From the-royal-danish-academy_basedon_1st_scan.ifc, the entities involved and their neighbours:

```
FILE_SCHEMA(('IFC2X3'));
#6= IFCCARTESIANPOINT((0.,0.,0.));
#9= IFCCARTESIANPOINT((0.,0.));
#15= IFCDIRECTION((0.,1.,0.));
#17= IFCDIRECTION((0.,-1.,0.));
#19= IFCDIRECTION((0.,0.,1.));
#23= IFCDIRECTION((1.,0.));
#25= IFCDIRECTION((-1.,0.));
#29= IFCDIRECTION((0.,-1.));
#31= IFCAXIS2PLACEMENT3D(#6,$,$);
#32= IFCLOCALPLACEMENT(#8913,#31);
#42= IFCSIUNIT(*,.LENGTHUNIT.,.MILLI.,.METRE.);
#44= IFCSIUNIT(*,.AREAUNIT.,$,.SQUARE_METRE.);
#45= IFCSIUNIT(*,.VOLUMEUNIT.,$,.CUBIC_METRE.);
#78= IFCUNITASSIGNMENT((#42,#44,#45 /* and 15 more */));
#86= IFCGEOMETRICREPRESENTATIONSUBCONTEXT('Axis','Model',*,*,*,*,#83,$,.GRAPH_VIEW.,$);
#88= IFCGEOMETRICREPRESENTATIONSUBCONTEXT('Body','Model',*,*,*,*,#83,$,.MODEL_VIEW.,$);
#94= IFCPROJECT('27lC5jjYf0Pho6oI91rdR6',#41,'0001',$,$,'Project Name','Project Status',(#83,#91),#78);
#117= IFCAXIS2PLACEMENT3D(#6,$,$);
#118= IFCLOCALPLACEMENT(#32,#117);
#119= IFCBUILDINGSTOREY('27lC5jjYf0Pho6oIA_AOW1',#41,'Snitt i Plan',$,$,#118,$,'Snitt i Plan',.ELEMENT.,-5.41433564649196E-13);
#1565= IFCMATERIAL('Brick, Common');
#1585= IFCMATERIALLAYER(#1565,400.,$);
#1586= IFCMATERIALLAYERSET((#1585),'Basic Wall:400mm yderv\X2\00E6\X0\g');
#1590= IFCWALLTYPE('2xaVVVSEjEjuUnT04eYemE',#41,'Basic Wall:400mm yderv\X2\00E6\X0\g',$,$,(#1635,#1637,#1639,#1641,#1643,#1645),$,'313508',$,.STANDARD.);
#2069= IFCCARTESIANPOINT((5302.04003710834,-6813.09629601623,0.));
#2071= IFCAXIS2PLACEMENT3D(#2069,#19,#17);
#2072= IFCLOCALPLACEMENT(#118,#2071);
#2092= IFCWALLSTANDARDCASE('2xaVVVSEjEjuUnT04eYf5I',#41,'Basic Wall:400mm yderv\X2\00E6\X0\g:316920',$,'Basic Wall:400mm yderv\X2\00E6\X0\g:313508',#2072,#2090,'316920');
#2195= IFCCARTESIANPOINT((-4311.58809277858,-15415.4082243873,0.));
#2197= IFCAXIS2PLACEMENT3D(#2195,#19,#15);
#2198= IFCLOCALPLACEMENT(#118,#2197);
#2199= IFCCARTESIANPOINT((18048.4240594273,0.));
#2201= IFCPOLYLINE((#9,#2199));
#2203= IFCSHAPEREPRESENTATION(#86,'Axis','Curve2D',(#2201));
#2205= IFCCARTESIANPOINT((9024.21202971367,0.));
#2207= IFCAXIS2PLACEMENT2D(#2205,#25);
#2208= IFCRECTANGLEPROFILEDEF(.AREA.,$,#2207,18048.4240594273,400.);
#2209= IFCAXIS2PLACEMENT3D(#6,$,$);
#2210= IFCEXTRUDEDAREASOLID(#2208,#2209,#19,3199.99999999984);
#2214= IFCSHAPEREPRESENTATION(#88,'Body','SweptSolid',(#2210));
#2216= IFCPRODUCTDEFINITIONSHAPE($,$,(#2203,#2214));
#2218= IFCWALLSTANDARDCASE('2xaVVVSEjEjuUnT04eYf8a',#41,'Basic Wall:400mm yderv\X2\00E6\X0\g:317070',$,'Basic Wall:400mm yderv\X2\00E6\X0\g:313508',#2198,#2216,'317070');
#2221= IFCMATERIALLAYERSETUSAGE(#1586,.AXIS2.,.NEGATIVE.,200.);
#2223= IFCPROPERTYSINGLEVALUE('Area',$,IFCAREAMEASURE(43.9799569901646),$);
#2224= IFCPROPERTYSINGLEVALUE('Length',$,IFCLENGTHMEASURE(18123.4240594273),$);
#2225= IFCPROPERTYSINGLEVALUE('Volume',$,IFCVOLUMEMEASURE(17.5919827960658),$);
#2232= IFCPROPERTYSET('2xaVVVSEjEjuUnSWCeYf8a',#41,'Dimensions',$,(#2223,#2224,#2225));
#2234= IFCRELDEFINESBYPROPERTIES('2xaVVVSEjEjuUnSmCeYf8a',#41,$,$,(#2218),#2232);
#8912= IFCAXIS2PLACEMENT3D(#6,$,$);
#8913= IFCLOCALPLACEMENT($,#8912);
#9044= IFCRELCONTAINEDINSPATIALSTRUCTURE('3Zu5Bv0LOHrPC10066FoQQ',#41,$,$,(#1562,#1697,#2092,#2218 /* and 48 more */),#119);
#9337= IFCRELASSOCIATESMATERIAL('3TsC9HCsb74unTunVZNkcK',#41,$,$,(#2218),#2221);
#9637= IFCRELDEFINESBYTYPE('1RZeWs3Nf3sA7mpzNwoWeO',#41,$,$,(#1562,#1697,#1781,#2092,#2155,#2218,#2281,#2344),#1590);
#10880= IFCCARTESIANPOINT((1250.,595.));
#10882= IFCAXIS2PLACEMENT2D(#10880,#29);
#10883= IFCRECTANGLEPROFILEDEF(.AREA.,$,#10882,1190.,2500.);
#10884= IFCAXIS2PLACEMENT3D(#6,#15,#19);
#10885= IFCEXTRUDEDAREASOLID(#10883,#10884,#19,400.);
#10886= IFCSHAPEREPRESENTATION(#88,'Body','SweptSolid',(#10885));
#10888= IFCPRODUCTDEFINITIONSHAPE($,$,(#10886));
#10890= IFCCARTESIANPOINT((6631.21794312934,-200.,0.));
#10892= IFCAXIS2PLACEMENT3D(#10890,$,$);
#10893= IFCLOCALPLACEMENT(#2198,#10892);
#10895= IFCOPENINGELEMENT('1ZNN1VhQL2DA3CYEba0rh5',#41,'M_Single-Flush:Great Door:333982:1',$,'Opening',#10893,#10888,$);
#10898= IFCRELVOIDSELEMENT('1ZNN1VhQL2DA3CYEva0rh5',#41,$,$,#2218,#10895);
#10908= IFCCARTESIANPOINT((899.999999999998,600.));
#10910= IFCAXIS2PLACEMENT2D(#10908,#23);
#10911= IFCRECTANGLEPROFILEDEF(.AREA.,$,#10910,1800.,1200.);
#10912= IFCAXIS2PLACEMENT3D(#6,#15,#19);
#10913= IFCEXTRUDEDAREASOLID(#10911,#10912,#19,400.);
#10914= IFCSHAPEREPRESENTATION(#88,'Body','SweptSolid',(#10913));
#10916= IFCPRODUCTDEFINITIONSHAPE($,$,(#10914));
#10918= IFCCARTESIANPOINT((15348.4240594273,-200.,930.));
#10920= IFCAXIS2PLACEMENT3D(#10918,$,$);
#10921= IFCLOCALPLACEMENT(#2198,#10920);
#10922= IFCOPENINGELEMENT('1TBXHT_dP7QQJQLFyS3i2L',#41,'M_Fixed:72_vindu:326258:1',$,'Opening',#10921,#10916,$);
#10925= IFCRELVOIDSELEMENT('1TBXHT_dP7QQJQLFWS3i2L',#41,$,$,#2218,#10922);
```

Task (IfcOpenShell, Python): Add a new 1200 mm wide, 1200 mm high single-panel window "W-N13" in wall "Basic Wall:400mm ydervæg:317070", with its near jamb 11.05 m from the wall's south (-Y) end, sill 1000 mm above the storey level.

```python
import numpy as np
import ifcopenshell
import ifcopenshell.api.feature
import ifcopenshell.api.geometry
import ifcopenshell.api.pset
import ifcopenshell.api.root
import ifcopenshell.api.spatial
import ifcopenshell.api.type
import ifcopenshell.geom
import ifcopenshell.util.element
import ifcopenshell.util.placement
import ifcopenshell.util.representation
import ifcopenshell.util.shape
import ifcopenshell.util.unit

model = ifcopenshell.open("the-royal-danish-academy_basedon_1st_scan.ifc")
unit_scale = ifcopenshell.util.unit.calculate_unit_scale(model)
area_scale = ifcopenshell.util.unit.calculate_unit_scale(model, "AREAUNIT")
volume_scale = ifcopenshell.util.unit.calculate_unit_scale(model, "VOLUMEUNIT")
settings = ifcopenshell.geom.settings()


def volume(element):
    """Net volume in cubic metres, openings subtracted."""
    shape = ifcopenshell.geom.create_shape(settings, element)
    return ifcopenshell.util.shape.get_volume(shape.geometry)


wall = model.by_guid("2xaVVVSEjEjuUnT04eYf8a")
storey = ifcopenshell.util.element.get_container(wall, ifc_class="IfcBuildingStorey")
context = ifcopenshell.util.representation.get_context(model, "Model", "Body", "MODEL_VIEW")
before = volume(wall)

width, height, from_end, sill = 1.2, 1.2, 11.05, 1  # metres

# The wall runs along its own X axis, and the end named is its -X end.
wall_shape = ifcopenshell.geom.create_shape(settings, wall)
x, y, z = ifcopenshell.util.shape.get_vertices(wall_shape.geometry).T
start = x.min() + from_end
face, thickness = float(y.min()), float(y.max() - y.min())
wall_matrix = ifcopenshell.util.placement.get_local_placement(wall.ObjectPlacement)
level = ifcopenshell.util.placement.get_local_placement(storey.ObjectPlacement)[2, 3]


def in_wall(x, y):
    """Placement at x, y metres in the wall's axes, at sill height."""
    matrix = wall_matrix.copy()
    matrix[:, 3] = wall_matrix @ np.array([x / unit_scale, y / unit_scale, 0.0, 1.0])
    matrix[2, 3] = level + sill / unit_scale
    return matrix


# Opening: a box that overshoots both wall faces by 50 mm.
opening = ifcopenshell.api.root.create_entity(model, ifc_class="IfcOpeningElement")
box = ifcopenshell.api.geometry.add_wall_representation(
    model, context=context, length=width, height=height, thickness=thickness + 0.1
)
ifcopenshell.api.geometry.assign_representation(model, product=opening, representation=box)
ifcopenshell.api.geometry.edit_object_placement(model, product=opening, matrix=in_wall(start, face - 0.05), is_si=False)
ifcopenshell.api.feature.add_feature(model, feature=opening, element=wall)

window = ifcopenshell.api.root.create_entity(model, ifc_class="IfcWindow", name="W-N13")
window.OverallWidth, window.OverallHeight = width / unit_scale, height / unit_scale
body = ifcopenshell.api.geometry.add_window_representation(
    model,
    context=context,
    overall_width=window.OverallWidth,
    overall_height=window.OverallHeight,
    partition_type="SINGLE_PANEL",
)
ifcopenshell.api.geometry.assign_representation(model, product=window, representation=body)
ifcopenshell.api.spatial.assign_container(model, products=[window], relating_structure=storey)
fills = ifcopenshell.api.feature.add_filling(model, opening=opening, element=window)
fills.OwnerHistory = window.OwnerHistory  # required in IFC2X3

# IFC2X3 keeps the operation on the window style.
style = ifcopenshell.api.root.create_entity(model, ifc_class="IfcWindowStyle", name="W-N13")
style.OperationType, style.ConstructionType = "SINGLE_PANEL", "NOTDEFINED"
style.ParameterTakesPrecedence = style.Sizeable = False
ifcopenshell.api.type.assign_type(model, related_objects=[window], relating_type=style)

# Centre the window in the wall's thickness.
ifcopenshell.api.geometry.edit_object_placement(model, product=window, matrix=in_wall(start, face), is_si=False)
window_shape = ifcopenshell.geom.create_shape(settings, window)
depth = ifcopenshell.util.shape.get_vertices(window_shape.geometry)[:, 1]
offset = face + thickness / 2 - (depth.min() + depth.max()) / 2
ifcopenshell.api.geometry.edit_object_placement(model, product=window, matrix=in_wall(start, offset), is_si=False)

after = volume(wall)

# Update the wall's stored quantities.
pset = model.by_id(ifcopenshell.util.element.get_pset(wall, "Dimensions", should_inherit=False)["id"])
ifcopenshell.api.pset.edit_pset(model, pset=pset, properties={
    "Area": model.create_entity("IfcAreaMeasure", after / thickness / area_scale),
    "Volume": model.create_entity("IfcVolumeMeasure", after / volume_scale),
})

print(f"wall volume {before:.3f} -> {after:.3f} m3")

model.write("the-royal-danish-academy_basedon_1st_scan_v2.ifc")
```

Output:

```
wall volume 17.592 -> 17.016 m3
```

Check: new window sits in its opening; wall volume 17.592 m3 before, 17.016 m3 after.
